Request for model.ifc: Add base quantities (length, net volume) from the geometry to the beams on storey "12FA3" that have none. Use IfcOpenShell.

First a look at what the model holds.

```python
import ifcopenshell
import ifcopenshell.util.element
import ifcopenshell.util.unit

model = ifcopenshell.open("model.ifc")
print(model.schema)
for unit_type in ("LENGTHUNIT", "AREAUNIT", "VOLUMEUNIT"):
    print(unit_type, ifcopenshell.util.unit.calculate_unit_scale(model, unit_type))
storey = next(s for s in model.by_type("IfcBuildingStorey") if s.Name == "12FA3")
beams = [e for e in ifcopenshell.util.element.get_decomposition(storey) if e.is_a("IfcBeam")]
for e in sorted(beams, key=lambda e: e.id()):
    print(e.id(), e.is_a(), e.Name, list(ifcopenshell.util.element.get_psets(e, qtos_only=True)), sep=" | ")
```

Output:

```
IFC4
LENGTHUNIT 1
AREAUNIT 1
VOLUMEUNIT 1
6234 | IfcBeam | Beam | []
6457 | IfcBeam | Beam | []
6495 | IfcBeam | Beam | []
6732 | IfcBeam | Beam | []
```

```python
import ifcopenshell
import ifcopenshell.api.pset
import ifcopenshell.geom
import ifcopenshell.util.element
import ifcopenshell.util.shape
import ifcopenshell.util.unit

model = ifcopenshell.open("model.ifc")
unit_scale = ifcopenshell.util.unit.calculate_unit_scale(model)
volume_scale = ifcopenshell.util.unit.calculate_unit_scale(model, "VOLUMEUNIT")
settings = ifcopenshell.geom.settings()

storey = next(s for s in model.by_type("IfcBuildingStorey") if s.Name == "12FA3")
beams = [e for e in ifcopenshell.util.element.get_decomposition(storey) if e.is_a("IfcBeam")]

for e in sorted(beams, key=lambda e: e.id()):
    if ifcopenshell.util.element.get_psets(e, qtos_only=True, should_inherit=False):
        continue
    # Geometry comes back in metres, in the element's own axes.
    shape = ifcopenshell.geom.create_shape(settings, e)
    values = {
        "Length": ifcopenshell.util.shape.get_max_xyz(shape.geometry) / unit_scale,
        "NetVolume": ifcopenshell.util.shape.get_volume(shape.geometry) / volume_scale,
    }
    qto = ifcopenshell.api.pset.add_qto(model, product=e, name="Qto_BeamBaseQuantities")
    ifcopenshell.api.pset.edit_qto(model, qto=qto, properties=values)
    print(e.id(), {k: round(v, 3) for k, v in values.items()})

model.write("model_v2.ifc")
```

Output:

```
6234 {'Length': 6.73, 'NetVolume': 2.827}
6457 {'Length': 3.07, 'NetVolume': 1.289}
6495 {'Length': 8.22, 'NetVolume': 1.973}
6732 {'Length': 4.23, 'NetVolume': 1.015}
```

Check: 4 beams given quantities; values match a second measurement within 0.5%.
